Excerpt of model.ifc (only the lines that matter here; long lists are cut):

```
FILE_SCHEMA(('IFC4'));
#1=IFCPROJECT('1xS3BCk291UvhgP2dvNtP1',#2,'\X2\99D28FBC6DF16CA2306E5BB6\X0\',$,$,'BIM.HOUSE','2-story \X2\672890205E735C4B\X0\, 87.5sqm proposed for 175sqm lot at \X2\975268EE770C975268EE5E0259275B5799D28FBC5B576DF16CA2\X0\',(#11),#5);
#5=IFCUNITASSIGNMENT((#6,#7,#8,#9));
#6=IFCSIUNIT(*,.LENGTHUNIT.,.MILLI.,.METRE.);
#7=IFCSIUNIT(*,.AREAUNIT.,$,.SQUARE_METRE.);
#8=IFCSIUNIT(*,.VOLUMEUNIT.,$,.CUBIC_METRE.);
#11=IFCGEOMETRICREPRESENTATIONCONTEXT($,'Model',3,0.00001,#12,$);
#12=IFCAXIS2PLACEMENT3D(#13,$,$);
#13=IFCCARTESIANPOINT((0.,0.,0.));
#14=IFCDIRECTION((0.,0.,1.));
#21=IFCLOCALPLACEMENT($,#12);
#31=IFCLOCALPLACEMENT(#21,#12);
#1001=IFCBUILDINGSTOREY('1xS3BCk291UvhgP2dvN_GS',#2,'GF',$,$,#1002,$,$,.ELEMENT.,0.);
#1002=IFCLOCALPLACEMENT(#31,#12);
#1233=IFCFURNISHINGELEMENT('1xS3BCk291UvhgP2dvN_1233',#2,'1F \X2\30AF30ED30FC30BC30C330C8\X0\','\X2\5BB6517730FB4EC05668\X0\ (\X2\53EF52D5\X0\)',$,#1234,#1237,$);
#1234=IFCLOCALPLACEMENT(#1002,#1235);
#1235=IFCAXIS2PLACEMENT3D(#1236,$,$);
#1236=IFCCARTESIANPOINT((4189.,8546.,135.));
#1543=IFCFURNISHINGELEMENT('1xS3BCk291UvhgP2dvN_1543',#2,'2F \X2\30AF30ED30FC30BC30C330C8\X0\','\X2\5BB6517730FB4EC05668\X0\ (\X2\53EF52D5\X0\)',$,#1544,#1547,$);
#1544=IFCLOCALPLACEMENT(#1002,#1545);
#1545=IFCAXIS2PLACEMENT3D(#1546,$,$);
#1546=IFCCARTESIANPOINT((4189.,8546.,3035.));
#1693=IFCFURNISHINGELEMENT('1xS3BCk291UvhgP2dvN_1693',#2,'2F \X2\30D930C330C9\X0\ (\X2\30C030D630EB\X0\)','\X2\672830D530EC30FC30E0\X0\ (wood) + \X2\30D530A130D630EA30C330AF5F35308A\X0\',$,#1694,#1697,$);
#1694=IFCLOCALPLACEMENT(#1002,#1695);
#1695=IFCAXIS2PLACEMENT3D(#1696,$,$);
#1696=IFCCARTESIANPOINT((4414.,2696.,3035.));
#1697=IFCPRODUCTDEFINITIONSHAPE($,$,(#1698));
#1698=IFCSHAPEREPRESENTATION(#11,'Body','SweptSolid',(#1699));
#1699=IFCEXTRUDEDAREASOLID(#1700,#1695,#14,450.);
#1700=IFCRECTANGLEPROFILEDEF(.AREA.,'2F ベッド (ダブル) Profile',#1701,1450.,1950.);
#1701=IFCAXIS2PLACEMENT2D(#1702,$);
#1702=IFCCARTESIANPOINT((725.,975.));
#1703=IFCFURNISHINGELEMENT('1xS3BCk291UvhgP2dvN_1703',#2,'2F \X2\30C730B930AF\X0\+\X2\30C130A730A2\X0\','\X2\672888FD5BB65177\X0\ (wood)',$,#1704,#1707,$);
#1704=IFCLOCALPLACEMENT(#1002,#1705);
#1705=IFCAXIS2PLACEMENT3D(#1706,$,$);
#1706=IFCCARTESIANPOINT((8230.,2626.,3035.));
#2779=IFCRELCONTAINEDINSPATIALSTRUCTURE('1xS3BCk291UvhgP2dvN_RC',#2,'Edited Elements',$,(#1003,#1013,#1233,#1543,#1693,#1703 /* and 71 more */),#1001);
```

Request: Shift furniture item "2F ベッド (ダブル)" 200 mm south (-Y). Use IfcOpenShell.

```python
import ifcopenshell
import ifcopenshell.api.geometry
import ifcopenshell.util.placement

model = ifcopenshell.open("model.ifc")

item = model.by_guid("1xS3BCk291UvhgP2dvN_1693")
matrix = ifcopenshell.util.placement.get_local_placement(item.ObjectPlacement)
matrix[1, 3] -= 200.0
ifcopenshell.api.geometry.edit_object_placement(model, product=item, matrix=matrix, is_si=False)

print(ifcopenshell.util.placement.get_local_placement(item.ObjectPlacement).round(3) + 0.0)

model.write("model_updated.ifc")
```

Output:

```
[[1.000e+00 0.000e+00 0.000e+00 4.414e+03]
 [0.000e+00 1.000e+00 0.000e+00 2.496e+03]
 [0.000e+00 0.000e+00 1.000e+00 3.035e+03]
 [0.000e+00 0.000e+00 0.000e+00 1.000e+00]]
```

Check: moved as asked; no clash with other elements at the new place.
